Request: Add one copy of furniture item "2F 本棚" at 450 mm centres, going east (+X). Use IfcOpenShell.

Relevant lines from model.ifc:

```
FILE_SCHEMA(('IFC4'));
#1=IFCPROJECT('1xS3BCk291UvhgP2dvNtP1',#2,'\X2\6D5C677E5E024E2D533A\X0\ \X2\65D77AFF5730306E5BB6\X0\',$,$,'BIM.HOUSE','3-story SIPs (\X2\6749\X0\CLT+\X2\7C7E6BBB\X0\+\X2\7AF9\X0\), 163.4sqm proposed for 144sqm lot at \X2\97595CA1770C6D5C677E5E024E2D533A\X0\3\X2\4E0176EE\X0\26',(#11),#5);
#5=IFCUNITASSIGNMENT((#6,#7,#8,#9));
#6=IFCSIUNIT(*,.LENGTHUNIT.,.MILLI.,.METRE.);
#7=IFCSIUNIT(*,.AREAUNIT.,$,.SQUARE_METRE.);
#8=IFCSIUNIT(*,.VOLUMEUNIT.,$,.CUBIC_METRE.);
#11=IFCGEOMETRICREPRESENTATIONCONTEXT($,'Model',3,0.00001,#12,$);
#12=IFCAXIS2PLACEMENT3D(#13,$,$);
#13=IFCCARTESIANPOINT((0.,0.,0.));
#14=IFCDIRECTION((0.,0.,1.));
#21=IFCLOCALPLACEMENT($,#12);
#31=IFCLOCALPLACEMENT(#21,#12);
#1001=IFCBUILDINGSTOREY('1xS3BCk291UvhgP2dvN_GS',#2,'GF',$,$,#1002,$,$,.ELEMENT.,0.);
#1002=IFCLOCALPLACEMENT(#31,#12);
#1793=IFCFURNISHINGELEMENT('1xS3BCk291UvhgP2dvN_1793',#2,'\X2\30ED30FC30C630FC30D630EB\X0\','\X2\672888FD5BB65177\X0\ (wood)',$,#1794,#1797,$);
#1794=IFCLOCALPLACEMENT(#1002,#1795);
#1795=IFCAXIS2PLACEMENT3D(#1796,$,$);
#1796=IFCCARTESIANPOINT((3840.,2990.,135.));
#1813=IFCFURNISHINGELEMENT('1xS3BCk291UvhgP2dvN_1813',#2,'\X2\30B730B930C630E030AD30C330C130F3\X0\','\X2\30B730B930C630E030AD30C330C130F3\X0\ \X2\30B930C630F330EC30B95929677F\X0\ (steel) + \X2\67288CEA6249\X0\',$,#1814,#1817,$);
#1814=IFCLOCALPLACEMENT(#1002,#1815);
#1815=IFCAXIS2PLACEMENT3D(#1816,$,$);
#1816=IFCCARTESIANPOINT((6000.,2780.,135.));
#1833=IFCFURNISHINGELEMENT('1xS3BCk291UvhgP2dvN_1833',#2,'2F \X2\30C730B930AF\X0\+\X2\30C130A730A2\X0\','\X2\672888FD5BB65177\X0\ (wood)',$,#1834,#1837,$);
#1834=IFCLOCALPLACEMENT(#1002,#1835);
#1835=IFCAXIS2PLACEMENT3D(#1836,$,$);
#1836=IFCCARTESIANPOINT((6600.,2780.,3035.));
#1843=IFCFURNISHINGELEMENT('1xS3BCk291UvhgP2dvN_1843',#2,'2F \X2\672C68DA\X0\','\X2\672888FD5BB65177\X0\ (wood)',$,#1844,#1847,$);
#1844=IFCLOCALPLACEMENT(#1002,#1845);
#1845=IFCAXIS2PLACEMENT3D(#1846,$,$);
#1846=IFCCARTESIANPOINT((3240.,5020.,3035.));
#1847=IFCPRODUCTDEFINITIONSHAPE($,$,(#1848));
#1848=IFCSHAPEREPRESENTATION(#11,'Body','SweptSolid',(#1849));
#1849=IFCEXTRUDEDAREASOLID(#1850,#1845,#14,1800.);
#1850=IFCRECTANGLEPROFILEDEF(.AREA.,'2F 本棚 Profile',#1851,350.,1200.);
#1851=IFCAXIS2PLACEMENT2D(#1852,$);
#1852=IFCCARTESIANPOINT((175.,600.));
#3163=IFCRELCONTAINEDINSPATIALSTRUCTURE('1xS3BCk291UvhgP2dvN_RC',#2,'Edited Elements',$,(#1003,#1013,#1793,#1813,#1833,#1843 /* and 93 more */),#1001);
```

```python
import numpy as np
import ifcopenshell
import ifcopenshell.api.geometry
import ifcopenshell.api.root
import ifcopenshell.util.element
import ifcopenshell.util.placement
import ifcopenshell.util.unit

model = ifcopenshell.open("model.ifc")
unit_scale = ifcopenshell.util.unit.calculate_unit_scale(model)


def reuse_history(source, copy):
    """copy_class also copies each property set's owner history, people and application; keep the originals."""
    for rel in copy.IsDefinedBy:
        if rel.is_a("IfcRelDefinesByProperties") and (history := rel.RelatingPropertyDefinition.OwnerHistory):
            rel.RelatingPropertyDefinition.OwnerHistory = source.OwnerHistory
            ifcopenshell.util.element.remove_deep2(model, history)


source = model.by_guid("1xS3BCk291UvhgP2dvN_1843")
base = ifcopenshell.util.placement.get_local_placement(source.ObjectPlacement)
step = np.array([1.0, 0.0, 0.0]) * 0.45 / unit_scale

for i in range(1, 2):
    copy = ifcopenshell.api.root.copy_class(model, product=source)
    copy.Representation = ifcopenshell.util.element.copy_deep(
        model, source.Representation, exclude=["IfcGeometricRepresentationContext", "IfcRepresentationMap"]
    )
    reuse_history(source, copy)
    matrix = base.copy()
    matrix[:3, 3] += i * step
    print("added at", matrix[:3, 3].round(3) + 0.0)
    ifcopenshell.api.geometry.edit_object_placement(model, product=copy, matrix=matrix, is_si=False)

model.write("model_edited.ifc")
```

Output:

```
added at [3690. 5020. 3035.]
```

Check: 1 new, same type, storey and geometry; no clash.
